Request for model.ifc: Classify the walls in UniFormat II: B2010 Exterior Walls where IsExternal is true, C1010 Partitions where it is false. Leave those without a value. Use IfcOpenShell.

First a look at what the model holds.

```python
import ifcopenshell
import ifcopenshell.util.element

model = ifcopenshell.open("model.ifc")
print(model.schema)
print("classifications:", [c.Name for c in model.by_type("IfcClassification")])
values = [ifcopenshell.util.element.get_pset(e, "Pset_WallCommon", "IsExternal") for e in model.by_type("IfcWall")]
for value in (True, False, None):
    print("IsExternal", value, values.count(value))
```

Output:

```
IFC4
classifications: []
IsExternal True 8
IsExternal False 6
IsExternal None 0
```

```python
import ifcopenshell
import ifcopenshell.api.classification
import ifcopenshell.util.element

model = ifcopenshell.open("model.ifc")

system = ifcopenshell.api.classification.add_classification(model, classification="UniFormat II")

walls = model.by_type("IfcWall")
external = {e: ifcopenshell.util.element.get_pset(e, "Pset_WallCommon", "IsExternal") for e in walls}
for flag, code, name in ((True, "B2010", "Exterior Walls"), (False, "C1010", "Partitions")):
    products = [e for e in walls if external[e] is flag]
    ifcopenshell.api.classification.add_reference(
        model, products=products, classification=system, identification=code, name=name
    )
    print(code, len(products))

model.write("model_rev.ifc")
```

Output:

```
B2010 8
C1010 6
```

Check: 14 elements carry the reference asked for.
